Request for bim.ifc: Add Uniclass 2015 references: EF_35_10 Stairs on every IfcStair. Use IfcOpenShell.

First a look at what the model holds.

```python
import ifcopenshell

model = ifcopenshell.open("bim.ifc")
print(model.schema)
print("classifications:", [c.Name for c in model.by_type("IfcClassification")])
for ifc_class in ("IfcDoor", "IfcRoof", "IfcStair", "IfcWall", "IfcWindow"):
    print(ifc_class, len(model.by_type(ifc_class)))
```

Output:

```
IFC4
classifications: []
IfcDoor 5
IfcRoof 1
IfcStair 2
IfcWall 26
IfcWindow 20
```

```python
import ifcopenshell
import ifcopenshell.api.classification

model = ifcopenshell.open("bim.ifc")

system = ifcopenshell.api.classification.add_classification(model, classification="Uniclass 2015")

codes = {
    "IfcStair": ("EF_35_10", "Stairs"),
}
for ifc_class, (code, name) in codes.items():
    products = model.by_type(ifc_class)
    ifcopenshell.api.classification.add_reference(
        model, products=products, classification=system, identification=code, name=name
    )
    print(code, len(products))

model.write("bim-out.ifc")
```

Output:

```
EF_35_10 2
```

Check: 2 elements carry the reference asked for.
